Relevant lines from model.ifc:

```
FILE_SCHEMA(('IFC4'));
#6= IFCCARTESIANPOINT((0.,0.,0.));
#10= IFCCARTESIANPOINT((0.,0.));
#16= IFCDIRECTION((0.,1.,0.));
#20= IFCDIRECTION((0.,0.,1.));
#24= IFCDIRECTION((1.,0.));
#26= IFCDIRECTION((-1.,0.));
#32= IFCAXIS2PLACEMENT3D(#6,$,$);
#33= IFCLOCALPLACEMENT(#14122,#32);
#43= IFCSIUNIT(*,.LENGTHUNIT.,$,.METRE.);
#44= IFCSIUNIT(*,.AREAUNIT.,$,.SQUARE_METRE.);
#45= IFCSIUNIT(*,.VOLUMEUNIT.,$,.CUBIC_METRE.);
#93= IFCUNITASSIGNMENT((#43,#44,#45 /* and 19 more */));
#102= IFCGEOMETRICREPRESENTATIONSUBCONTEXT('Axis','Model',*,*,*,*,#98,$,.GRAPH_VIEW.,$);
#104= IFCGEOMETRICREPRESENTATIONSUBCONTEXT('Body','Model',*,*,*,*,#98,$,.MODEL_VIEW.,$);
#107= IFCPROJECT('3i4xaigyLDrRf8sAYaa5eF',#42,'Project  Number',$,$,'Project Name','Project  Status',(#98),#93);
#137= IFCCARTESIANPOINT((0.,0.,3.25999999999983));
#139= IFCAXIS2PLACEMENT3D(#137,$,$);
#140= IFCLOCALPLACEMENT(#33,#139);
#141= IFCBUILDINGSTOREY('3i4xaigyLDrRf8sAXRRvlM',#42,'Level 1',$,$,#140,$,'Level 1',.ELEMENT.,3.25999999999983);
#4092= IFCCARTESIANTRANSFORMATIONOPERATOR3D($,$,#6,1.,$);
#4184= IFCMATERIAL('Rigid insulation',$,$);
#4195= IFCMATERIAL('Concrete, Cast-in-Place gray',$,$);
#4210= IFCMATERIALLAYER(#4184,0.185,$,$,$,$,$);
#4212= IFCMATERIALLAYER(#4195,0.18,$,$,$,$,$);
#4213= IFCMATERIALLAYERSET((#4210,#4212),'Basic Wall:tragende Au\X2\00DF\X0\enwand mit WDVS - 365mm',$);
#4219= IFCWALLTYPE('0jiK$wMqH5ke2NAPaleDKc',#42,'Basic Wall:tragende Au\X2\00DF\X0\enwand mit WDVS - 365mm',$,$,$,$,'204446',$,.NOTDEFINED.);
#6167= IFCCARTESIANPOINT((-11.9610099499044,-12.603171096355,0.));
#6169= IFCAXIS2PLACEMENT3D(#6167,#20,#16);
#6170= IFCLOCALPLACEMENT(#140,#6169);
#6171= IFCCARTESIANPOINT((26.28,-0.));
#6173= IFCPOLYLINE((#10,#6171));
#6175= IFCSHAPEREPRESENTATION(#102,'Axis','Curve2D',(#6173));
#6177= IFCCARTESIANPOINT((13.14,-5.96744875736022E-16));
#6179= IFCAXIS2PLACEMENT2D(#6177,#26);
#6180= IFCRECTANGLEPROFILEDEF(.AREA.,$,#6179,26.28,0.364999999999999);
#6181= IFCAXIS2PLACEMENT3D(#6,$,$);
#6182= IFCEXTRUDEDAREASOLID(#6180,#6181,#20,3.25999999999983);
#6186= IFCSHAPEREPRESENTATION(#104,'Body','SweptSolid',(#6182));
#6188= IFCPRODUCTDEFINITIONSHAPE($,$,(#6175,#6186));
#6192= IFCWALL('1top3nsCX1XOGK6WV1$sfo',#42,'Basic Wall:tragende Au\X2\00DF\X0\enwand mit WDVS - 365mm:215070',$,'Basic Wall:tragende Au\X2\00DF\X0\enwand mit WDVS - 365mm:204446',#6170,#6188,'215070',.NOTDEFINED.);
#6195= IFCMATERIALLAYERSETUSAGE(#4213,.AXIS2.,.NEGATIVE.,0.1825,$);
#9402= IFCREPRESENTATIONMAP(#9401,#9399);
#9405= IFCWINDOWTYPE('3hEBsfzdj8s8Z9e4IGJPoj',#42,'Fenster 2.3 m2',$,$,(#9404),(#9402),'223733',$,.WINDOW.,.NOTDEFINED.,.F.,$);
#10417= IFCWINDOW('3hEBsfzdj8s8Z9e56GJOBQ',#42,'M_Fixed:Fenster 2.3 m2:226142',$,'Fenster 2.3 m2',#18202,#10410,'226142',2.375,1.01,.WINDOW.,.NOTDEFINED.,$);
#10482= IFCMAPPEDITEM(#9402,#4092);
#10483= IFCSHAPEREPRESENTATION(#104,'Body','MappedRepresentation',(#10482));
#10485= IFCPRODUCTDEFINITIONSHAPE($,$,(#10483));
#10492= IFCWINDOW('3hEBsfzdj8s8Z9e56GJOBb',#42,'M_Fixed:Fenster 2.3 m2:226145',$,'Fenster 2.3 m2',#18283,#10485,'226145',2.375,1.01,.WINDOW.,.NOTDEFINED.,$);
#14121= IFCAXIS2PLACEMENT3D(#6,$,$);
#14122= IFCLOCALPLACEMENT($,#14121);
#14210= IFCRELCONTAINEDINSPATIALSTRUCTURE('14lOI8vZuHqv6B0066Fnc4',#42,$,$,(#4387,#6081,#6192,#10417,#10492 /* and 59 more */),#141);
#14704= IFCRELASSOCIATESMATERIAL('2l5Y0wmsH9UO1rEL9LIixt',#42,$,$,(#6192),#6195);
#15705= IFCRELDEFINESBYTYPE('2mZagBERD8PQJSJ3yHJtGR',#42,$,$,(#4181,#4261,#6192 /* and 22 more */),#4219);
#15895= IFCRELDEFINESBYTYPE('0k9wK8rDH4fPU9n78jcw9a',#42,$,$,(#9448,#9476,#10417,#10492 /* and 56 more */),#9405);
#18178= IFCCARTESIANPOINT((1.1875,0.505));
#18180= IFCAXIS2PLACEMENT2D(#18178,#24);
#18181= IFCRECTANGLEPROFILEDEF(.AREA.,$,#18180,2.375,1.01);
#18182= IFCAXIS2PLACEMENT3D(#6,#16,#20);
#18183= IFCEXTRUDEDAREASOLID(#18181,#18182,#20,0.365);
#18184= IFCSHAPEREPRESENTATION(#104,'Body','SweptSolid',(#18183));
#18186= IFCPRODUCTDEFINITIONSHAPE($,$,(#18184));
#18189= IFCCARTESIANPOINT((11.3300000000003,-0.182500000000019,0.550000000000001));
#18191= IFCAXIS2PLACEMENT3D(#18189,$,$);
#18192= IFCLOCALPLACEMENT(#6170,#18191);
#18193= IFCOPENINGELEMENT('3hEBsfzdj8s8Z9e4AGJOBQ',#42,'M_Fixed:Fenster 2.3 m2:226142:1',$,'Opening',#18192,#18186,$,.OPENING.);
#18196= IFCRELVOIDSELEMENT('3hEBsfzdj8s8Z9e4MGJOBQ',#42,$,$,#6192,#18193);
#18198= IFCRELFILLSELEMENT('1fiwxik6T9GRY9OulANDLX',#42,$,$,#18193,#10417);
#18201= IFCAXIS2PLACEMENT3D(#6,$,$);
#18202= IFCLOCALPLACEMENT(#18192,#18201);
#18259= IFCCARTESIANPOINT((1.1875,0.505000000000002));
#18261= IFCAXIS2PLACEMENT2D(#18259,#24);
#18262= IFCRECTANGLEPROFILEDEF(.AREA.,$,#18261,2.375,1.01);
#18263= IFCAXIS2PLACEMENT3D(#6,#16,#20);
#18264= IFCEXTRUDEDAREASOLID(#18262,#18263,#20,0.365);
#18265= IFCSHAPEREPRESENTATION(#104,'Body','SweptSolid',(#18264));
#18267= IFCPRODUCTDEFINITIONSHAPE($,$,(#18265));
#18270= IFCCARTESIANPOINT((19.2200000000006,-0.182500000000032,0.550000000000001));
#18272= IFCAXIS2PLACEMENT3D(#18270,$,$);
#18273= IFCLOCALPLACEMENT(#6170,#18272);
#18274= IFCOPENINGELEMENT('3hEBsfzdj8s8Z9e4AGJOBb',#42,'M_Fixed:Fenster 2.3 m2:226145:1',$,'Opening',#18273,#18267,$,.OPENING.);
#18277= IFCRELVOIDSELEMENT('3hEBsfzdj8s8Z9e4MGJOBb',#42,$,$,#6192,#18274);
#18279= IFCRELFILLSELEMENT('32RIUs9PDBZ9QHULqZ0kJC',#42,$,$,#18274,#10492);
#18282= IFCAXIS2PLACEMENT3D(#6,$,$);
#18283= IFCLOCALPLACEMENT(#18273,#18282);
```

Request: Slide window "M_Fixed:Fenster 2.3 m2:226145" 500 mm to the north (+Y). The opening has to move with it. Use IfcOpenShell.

```python
import ifcopenshell
import ifcopenshell.api.geometry
import ifcopenshell.util.placement
import ifcopenshell.util.unit

model = ifcopenshell.open("model.ifc")
unit_scale = ifcopenshell.util.unit.calculate_unit_scale(model)

window = model.by_id(10492)
opening = window.FillsVoids[0].RelatingOpeningElement
wall = opening.VoidsElements[0].RelatingBuildingElement

wall_matrix = ifcopenshell.util.placement.get_local_placement(wall.ObjectPlacement)
shift = wall_matrix[:3, 0] * 0.5 / unit_scale
before = ifcopenshell.util.placement.get_local_placement(window.ObjectPlacement)[:3, 3].copy()

# The window is placed relative to its opening, so it follows when the opening moves.
matrix = ifcopenshell.util.placement.get_local_placement(opening.ObjectPlacement)
matrix[:3, 3] += shift
ifcopenshell.api.geometry.edit_object_placement(
    model, product=opening, matrix=matrix, is_si=False, should_transform_children=True
)

after = ifcopenshell.util.placement.get_local_placement(window.ObjectPlacement)[:3, 3]
print("window moved by", (after - before).round(3) + 0.0)

model.write("model-out.ifc")
```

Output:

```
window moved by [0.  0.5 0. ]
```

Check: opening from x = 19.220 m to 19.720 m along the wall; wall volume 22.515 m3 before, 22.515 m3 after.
